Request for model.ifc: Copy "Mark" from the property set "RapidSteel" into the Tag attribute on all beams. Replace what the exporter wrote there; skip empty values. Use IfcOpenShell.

First a look at what the model holds.

```python
import ifcopenshell
import ifcopenshell.util.element

model = ifcopenshell.open("model.ifc")
print(model.schema)
beams = model.by_type("IfcBeam")
print(len(beams), "beams")
for e in beams[:8]:
    source = ifcopenshell.util.element.get_pset(e, "RapidSteel", "Mark")
    target = e.Tag
    print(e.id(), repr(source), repr(target), sep=" | ")
```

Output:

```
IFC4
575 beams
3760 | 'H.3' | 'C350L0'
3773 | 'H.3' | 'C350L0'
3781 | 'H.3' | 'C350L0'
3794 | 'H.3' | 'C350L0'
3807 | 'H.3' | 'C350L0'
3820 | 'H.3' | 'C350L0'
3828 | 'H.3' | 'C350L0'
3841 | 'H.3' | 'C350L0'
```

```python
import ifcopenshell
import ifcopenshell.util.element

model = ifcopenshell.open("model.ifc")

count = 0
for e in model.by_type("IfcBeam"):
    value = ifcopenshell.util.element.get_pset(e, "RapidSteel", "Mark")
    current = e.Tag
    if not value or not value.strip() or current == value:
        continue
    e.Tag = value
    count += 1

print(count, "beams updated")

model.write("model_v2.ifc")
```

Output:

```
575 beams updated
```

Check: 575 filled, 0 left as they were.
